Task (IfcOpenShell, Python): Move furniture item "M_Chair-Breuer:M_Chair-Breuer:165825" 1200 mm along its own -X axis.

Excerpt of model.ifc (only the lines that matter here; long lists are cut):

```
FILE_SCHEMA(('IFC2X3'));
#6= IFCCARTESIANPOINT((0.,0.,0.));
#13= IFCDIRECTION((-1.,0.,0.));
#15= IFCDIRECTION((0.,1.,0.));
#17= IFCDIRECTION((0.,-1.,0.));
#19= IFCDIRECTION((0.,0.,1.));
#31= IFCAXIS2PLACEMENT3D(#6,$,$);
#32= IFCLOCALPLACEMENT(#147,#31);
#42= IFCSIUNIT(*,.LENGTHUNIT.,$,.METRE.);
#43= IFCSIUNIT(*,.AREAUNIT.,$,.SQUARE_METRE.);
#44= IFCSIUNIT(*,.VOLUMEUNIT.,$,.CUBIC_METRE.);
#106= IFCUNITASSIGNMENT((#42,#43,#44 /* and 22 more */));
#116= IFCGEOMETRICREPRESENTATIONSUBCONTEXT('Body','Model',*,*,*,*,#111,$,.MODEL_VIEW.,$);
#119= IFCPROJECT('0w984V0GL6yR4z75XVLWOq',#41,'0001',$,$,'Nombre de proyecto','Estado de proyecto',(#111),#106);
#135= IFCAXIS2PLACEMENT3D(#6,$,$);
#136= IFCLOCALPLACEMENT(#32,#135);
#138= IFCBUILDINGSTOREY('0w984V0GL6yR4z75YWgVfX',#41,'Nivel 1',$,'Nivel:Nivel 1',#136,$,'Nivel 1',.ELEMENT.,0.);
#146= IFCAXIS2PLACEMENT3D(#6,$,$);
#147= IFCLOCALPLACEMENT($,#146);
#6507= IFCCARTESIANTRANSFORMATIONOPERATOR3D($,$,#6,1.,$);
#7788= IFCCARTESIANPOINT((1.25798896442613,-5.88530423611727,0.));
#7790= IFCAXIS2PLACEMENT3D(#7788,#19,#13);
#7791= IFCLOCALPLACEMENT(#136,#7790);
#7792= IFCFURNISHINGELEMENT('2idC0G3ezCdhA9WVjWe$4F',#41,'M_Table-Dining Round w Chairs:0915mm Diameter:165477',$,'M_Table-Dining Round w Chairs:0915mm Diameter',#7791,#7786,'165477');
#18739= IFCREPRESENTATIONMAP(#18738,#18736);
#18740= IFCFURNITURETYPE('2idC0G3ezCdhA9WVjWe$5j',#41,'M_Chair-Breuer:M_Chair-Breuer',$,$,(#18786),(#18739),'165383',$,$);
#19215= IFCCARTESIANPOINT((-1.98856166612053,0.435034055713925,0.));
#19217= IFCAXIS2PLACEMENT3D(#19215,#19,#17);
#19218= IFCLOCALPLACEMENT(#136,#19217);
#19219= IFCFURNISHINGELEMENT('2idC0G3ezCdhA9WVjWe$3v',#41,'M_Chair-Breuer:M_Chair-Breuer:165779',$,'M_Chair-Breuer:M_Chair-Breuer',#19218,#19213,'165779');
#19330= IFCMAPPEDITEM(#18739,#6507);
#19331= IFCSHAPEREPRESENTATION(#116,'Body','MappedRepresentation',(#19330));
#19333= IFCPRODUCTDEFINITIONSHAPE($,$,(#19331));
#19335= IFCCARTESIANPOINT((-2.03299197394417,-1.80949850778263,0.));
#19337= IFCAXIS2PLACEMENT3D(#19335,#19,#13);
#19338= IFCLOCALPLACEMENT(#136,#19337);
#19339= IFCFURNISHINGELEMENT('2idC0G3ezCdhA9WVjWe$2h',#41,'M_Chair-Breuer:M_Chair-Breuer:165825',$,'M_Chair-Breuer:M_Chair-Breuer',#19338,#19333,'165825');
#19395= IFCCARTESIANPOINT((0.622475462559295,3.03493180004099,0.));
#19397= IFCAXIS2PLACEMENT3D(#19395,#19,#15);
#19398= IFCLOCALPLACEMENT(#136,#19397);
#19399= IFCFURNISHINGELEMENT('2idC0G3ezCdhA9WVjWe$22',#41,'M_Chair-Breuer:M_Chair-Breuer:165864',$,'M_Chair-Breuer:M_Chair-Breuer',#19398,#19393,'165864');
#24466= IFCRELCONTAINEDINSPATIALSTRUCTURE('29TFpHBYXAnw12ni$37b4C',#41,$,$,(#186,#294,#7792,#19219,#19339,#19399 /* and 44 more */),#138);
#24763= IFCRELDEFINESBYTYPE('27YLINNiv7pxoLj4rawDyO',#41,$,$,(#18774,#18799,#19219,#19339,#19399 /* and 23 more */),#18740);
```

```python
import ifcopenshell
import ifcopenshell.api.geometry
import ifcopenshell.util.placement
import ifcopenshell.util.unit

model = ifcopenshell.open("model.ifc")
unit_scale = ifcopenshell.util.unit.calculate_unit_scale(model)

item = model.by_id(19339)
matrix = ifcopenshell.util.placement.get_local_placement(item.ObjectPlacement)
matrix[:3, 3] -= matrix[:3, 0] * 1.2 / unit_scale
ifcopenshell.api.geometry.edit_object_placement(model, product=item, matrix=matrix, is_si=False)

print(ifcopenshell.util.placement.get_local_placement(item.ObjectPlacement).round(3) + 0.0)

model.write("model_v2.ifc")
```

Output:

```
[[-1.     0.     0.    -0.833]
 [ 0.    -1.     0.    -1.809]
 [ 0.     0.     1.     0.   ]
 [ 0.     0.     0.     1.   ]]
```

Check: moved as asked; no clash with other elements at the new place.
